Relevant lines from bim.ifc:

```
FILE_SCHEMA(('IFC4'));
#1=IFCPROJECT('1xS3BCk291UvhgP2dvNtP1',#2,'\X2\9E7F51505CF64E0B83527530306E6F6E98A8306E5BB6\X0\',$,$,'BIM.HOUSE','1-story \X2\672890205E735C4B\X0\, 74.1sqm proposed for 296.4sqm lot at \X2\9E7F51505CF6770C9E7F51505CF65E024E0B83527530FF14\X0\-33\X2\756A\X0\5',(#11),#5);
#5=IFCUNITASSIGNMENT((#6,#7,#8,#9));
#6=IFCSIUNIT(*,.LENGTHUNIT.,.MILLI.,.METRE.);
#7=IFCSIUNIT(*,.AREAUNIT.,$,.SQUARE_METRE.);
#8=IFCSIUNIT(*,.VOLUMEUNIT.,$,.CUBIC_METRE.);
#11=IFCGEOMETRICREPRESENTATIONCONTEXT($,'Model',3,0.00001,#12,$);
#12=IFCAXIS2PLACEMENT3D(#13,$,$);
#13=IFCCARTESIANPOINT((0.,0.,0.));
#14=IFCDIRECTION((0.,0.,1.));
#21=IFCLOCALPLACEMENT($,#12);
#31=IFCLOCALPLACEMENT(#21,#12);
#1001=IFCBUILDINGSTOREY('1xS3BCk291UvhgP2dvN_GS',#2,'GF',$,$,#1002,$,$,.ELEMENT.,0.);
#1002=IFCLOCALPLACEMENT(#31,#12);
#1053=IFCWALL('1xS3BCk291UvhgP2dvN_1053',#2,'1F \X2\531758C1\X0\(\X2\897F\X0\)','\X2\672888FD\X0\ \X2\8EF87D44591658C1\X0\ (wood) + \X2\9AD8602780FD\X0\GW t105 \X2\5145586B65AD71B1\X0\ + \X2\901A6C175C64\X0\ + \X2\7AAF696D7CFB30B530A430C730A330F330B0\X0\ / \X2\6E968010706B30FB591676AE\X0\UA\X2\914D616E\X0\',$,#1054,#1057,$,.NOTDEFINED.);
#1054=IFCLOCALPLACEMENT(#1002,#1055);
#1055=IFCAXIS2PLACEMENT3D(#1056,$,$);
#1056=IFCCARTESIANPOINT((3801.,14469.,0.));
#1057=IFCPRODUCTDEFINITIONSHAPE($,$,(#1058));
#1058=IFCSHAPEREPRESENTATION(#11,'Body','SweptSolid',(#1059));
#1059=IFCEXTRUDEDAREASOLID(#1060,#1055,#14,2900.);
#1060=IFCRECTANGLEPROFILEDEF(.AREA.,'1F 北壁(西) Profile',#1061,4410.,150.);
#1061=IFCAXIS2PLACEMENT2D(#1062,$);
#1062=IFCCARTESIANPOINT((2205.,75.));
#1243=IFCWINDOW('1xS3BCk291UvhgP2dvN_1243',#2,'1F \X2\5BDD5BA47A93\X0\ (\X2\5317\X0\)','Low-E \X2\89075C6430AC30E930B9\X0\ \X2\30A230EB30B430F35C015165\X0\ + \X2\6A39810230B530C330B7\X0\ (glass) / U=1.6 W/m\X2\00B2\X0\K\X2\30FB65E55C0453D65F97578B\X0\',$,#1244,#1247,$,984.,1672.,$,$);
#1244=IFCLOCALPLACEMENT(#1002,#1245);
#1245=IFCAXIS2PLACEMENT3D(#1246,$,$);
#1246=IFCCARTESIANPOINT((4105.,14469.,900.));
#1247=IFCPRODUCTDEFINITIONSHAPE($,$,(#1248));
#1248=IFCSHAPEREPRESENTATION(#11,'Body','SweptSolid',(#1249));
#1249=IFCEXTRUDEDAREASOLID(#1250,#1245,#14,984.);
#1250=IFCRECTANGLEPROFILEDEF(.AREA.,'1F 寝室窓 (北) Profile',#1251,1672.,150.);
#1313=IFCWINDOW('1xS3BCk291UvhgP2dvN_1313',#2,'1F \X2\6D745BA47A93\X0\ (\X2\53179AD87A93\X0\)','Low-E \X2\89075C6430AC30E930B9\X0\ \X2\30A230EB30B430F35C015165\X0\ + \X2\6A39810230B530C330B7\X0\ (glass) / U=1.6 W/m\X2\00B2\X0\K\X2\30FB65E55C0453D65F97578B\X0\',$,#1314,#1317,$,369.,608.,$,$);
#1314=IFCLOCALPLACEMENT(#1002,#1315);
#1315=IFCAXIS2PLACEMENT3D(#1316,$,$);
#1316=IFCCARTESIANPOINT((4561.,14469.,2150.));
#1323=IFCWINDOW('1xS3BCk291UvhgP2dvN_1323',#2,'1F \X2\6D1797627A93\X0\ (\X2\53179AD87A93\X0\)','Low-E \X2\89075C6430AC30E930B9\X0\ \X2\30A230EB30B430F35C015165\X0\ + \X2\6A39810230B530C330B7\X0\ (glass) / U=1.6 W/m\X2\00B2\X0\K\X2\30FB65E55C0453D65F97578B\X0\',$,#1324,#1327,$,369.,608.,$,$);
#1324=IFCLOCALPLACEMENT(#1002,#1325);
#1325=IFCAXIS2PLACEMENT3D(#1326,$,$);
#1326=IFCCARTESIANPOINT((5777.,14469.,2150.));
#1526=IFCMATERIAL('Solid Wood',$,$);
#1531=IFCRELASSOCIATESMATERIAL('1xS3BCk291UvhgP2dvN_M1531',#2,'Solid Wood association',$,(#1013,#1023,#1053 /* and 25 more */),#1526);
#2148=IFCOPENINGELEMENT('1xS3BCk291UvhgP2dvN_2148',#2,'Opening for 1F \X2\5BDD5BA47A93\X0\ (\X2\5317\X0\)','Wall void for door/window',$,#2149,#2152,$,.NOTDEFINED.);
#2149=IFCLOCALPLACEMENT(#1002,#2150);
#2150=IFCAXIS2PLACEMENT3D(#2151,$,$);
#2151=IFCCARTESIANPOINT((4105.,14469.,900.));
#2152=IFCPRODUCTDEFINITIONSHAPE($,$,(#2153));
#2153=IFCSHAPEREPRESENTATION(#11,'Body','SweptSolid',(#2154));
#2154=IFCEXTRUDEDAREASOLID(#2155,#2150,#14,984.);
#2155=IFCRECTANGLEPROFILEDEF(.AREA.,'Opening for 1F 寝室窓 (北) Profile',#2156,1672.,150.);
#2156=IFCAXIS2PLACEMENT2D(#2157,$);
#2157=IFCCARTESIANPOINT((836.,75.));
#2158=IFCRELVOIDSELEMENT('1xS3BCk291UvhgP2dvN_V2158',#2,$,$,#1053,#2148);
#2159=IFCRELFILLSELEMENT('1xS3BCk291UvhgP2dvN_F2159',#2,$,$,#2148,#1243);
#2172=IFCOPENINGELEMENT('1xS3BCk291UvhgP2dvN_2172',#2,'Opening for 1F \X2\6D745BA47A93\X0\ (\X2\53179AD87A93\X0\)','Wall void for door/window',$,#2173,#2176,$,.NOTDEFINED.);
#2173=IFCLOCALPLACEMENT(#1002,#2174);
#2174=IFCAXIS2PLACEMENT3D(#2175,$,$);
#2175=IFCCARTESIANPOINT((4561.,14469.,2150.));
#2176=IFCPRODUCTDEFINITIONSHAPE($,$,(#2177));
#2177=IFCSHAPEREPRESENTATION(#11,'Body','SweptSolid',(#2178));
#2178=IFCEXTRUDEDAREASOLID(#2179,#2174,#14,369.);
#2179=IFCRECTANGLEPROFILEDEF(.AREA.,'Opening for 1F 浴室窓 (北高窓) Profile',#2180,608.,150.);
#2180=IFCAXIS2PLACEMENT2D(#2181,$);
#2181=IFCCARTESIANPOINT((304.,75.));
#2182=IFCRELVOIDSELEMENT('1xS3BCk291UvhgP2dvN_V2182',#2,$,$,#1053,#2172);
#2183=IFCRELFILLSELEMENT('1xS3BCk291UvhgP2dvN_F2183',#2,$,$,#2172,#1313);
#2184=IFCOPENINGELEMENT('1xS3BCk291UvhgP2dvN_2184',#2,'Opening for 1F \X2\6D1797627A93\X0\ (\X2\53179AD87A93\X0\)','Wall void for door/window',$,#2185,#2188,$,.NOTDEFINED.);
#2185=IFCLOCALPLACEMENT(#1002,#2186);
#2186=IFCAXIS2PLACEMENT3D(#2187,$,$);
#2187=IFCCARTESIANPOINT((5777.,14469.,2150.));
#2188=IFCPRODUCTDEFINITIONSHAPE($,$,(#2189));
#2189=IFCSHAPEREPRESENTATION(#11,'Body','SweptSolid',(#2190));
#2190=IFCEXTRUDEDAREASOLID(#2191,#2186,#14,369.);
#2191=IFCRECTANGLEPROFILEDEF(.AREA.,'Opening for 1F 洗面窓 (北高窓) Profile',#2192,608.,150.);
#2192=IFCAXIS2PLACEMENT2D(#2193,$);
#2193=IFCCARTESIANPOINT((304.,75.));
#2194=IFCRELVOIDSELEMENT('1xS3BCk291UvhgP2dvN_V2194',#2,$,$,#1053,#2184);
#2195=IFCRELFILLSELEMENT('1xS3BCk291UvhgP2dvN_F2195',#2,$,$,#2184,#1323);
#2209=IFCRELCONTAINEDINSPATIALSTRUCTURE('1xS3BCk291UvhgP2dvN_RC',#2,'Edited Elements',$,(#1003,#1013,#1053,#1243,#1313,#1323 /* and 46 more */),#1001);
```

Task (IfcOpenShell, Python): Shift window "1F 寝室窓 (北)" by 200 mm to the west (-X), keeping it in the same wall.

```python
import ifcopenshell
import ifcopenshell.api.geometry
import ifcopenshell.util.placement
import ifcopenshell.util.unit

model = ifcopenshell.open("bim.ifc")
unit_scale = ifcopenshell.util.unit.calculate_unit_scale(model)

window = model.by_id(1243)
opening = window.FillsVoids[0].RelatingOpeningElement
wall = opening.VoidsElements[0].RelatingBuildingElement

wall_matrix = ifcopenshell.util.placement.get_local_placement(wall.ObjectPlacement)
shift = wall_matrix[:3, 0] * -0.2 / unit_scale
before = ifcopenshell.util.placement.get_local_placement(window.ObjectPlacement)[:3, 3].copy()

# The window is not placed relative to its opening, so move both.
for product in (opening, window):
    matrix = ifcopenshell.util.placement.get_local_placement(product.ObjectPlacement)
    matrix[:3, 3] += shift
    ifcopenshell.api.geometry.edit_object_placement(model, product=product, matrix=matrix, is_si=False)

after = ifcopenshell.util.placement.get_local_placement(window.ObjectPlacement)[:3, 3]
print("window moved by", (after - before).round(3) + 0.0)

model.write("bim_updated.ifc")
```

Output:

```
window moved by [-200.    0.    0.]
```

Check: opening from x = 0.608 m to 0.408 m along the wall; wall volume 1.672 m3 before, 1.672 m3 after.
